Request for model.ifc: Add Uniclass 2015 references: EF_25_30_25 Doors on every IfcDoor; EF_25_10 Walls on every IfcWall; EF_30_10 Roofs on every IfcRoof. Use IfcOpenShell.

First a look at what the model holds.

```python
import ifcopenshell

model = ifcopenshell.open("model.ifc")
print(model.schema)
print("classifications:", [c.Name for c in model.by_type("IfcClassification")])
for ifc_class in ("IfcDoor", "IfcRoof", "IfcStair", "IfcWall", "IfcWindow"):
    print(ifc_class, len(model.by_type(ifc_class)))
```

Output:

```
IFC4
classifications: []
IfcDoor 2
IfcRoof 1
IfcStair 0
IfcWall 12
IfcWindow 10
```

```python
import ifcopenshell
import ifcopenshell.api.classification

model = ifcopenshell.open("model.ifc")

system = ifcopenshell.api.classification.add_classification(model, classification="Uniclass 2015")

codes = {
    "IfcDoor": ("EF_25_30_25", "Doors"),
    "IfcWall": ("EF_25_10", "Walls"),
    "IfcRoof": ("EF_30_10", "Roofs"),
}
for ifc_class, (code, name) in codes.items():
    products = model.by_type(ifc_class)
    ifcopenshell.api.classification.add_reference(
        model, products=products, classification=system, identification=code, name=name
    )
    print(code, len(products))

model.write("model_updated.ifc")
```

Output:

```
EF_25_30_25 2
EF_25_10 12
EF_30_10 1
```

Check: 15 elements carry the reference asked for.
